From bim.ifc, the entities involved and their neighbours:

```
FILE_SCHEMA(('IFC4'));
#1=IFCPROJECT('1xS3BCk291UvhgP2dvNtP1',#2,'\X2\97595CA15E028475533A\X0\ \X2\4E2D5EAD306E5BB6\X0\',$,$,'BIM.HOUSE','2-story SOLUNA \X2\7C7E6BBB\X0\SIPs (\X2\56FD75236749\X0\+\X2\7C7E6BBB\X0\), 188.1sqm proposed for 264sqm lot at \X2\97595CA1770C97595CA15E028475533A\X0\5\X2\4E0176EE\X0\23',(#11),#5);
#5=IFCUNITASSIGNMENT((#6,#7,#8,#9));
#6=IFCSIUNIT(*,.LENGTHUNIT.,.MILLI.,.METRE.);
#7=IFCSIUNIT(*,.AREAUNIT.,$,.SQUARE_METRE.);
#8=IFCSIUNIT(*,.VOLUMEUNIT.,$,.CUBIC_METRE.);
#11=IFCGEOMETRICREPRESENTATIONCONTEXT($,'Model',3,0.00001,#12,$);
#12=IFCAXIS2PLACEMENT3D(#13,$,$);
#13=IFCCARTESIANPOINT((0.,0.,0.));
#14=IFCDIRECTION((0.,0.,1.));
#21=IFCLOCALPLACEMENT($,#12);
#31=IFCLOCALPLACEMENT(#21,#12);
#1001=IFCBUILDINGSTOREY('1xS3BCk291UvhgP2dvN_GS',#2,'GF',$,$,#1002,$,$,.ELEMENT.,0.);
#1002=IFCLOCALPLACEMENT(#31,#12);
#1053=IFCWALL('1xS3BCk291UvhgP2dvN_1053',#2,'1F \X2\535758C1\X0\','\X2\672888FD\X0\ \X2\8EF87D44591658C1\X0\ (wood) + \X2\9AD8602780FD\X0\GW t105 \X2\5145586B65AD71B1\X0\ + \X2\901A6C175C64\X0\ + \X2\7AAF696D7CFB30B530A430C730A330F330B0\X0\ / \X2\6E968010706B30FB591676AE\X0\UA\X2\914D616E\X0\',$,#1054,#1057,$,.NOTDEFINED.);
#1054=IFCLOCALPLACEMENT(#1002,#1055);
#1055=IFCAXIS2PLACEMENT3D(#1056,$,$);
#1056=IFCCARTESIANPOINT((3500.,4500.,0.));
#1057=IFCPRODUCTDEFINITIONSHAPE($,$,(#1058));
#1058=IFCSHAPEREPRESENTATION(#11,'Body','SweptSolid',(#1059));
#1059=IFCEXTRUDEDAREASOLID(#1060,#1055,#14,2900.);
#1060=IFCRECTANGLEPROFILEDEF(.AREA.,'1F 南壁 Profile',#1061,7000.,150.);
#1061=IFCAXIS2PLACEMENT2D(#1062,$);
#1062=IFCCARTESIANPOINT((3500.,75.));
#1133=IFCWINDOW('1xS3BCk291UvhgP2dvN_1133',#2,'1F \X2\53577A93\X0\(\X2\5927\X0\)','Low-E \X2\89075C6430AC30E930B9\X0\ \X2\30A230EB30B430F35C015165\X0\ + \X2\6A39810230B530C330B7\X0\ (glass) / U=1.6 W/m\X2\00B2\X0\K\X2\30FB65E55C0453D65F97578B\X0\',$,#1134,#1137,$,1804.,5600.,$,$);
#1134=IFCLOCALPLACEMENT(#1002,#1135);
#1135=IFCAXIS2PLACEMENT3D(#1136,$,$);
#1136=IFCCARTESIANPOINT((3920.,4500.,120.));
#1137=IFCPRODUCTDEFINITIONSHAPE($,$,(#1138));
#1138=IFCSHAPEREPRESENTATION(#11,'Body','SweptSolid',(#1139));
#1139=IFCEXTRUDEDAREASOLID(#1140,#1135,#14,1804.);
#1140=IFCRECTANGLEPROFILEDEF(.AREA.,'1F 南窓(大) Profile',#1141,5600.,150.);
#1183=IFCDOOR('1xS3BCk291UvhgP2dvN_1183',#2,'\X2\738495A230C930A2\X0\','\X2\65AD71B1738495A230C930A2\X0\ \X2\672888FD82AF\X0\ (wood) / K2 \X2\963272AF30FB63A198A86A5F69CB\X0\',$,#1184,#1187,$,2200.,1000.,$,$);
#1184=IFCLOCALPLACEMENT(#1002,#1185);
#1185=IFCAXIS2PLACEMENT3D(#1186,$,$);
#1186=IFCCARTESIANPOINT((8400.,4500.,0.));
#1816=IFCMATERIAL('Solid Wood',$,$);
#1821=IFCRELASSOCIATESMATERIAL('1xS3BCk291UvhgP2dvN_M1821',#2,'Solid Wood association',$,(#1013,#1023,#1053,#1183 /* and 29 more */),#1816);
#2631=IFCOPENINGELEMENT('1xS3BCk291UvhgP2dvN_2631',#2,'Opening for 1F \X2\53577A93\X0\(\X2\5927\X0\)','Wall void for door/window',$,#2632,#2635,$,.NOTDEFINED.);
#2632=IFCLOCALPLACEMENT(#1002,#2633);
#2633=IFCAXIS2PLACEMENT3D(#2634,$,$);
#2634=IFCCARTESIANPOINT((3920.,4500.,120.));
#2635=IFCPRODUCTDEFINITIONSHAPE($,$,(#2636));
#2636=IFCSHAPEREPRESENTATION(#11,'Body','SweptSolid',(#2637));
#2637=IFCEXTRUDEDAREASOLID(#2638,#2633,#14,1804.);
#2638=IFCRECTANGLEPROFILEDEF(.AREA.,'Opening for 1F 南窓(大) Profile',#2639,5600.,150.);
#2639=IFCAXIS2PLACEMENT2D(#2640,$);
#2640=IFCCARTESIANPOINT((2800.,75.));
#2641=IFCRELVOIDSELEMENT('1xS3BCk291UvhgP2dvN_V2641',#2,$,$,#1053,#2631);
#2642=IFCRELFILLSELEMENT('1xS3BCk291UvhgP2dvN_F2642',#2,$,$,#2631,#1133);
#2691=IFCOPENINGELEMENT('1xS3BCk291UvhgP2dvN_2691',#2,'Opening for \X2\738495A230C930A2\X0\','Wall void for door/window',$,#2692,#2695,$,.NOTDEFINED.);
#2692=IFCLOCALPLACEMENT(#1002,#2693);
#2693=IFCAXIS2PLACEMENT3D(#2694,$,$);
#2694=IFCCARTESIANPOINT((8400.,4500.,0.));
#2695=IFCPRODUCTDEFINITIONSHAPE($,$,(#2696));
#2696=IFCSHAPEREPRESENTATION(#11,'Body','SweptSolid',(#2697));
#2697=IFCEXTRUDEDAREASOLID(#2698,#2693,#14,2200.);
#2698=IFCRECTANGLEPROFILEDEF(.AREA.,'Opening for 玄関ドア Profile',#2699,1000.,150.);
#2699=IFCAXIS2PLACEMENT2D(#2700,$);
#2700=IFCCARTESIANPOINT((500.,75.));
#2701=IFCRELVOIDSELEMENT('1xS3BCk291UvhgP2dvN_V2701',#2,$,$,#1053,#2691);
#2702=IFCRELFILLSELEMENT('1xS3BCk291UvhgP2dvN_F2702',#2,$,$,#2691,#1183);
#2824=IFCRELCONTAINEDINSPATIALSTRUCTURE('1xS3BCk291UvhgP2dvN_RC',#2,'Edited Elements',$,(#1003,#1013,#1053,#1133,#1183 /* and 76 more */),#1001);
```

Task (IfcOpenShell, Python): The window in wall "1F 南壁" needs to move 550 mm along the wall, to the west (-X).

```python
import ifcopenshell
import ifcopenshell.api.geometry
import ifcopenshell.util.placement
import ifcopenshell.util.unit

model = ifcopenshell.open("bim.ifc")
unit_scale = ifcopenshell.util.unit.calculate_unit_scale(model)

window = model.by_id(1133)
opening = window.FillsVoids[0].RelatingOpeningElement
wall = opening.VoidsElements[0].RelatingBuildingElement

wall_matrix = ifcopenshell.util.placement.get_local_placement(wall.ObjectPlacement)
shift = wall_matrix[:3, 0] * -0.55 / unit_scale
before = ifcopenshell.util.placement.get_local_placement(window.ObjectPlacement)[:3, 3].copy()

# The window is not placed relative to its opening, so move both.
for product in (opening, window):
    matrix = ifcopenshell.util.placement.get_local_placement(product.ObjectPlacement)
    matrix[:3, 3] += shift
    ifcopenshell.api.geometry.edit_object_placement(model, product=product, matrix=matrix, is_si=False)

after = ifcopenshell.util.placement.get_local_placement(window.ObjectPlacement)[:3, 3]
print("window moved by", (after - before).round(3) + 0.0)

model.write("bim-out.ifc")
```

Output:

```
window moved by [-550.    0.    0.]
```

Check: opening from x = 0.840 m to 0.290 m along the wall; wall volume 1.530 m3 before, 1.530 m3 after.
